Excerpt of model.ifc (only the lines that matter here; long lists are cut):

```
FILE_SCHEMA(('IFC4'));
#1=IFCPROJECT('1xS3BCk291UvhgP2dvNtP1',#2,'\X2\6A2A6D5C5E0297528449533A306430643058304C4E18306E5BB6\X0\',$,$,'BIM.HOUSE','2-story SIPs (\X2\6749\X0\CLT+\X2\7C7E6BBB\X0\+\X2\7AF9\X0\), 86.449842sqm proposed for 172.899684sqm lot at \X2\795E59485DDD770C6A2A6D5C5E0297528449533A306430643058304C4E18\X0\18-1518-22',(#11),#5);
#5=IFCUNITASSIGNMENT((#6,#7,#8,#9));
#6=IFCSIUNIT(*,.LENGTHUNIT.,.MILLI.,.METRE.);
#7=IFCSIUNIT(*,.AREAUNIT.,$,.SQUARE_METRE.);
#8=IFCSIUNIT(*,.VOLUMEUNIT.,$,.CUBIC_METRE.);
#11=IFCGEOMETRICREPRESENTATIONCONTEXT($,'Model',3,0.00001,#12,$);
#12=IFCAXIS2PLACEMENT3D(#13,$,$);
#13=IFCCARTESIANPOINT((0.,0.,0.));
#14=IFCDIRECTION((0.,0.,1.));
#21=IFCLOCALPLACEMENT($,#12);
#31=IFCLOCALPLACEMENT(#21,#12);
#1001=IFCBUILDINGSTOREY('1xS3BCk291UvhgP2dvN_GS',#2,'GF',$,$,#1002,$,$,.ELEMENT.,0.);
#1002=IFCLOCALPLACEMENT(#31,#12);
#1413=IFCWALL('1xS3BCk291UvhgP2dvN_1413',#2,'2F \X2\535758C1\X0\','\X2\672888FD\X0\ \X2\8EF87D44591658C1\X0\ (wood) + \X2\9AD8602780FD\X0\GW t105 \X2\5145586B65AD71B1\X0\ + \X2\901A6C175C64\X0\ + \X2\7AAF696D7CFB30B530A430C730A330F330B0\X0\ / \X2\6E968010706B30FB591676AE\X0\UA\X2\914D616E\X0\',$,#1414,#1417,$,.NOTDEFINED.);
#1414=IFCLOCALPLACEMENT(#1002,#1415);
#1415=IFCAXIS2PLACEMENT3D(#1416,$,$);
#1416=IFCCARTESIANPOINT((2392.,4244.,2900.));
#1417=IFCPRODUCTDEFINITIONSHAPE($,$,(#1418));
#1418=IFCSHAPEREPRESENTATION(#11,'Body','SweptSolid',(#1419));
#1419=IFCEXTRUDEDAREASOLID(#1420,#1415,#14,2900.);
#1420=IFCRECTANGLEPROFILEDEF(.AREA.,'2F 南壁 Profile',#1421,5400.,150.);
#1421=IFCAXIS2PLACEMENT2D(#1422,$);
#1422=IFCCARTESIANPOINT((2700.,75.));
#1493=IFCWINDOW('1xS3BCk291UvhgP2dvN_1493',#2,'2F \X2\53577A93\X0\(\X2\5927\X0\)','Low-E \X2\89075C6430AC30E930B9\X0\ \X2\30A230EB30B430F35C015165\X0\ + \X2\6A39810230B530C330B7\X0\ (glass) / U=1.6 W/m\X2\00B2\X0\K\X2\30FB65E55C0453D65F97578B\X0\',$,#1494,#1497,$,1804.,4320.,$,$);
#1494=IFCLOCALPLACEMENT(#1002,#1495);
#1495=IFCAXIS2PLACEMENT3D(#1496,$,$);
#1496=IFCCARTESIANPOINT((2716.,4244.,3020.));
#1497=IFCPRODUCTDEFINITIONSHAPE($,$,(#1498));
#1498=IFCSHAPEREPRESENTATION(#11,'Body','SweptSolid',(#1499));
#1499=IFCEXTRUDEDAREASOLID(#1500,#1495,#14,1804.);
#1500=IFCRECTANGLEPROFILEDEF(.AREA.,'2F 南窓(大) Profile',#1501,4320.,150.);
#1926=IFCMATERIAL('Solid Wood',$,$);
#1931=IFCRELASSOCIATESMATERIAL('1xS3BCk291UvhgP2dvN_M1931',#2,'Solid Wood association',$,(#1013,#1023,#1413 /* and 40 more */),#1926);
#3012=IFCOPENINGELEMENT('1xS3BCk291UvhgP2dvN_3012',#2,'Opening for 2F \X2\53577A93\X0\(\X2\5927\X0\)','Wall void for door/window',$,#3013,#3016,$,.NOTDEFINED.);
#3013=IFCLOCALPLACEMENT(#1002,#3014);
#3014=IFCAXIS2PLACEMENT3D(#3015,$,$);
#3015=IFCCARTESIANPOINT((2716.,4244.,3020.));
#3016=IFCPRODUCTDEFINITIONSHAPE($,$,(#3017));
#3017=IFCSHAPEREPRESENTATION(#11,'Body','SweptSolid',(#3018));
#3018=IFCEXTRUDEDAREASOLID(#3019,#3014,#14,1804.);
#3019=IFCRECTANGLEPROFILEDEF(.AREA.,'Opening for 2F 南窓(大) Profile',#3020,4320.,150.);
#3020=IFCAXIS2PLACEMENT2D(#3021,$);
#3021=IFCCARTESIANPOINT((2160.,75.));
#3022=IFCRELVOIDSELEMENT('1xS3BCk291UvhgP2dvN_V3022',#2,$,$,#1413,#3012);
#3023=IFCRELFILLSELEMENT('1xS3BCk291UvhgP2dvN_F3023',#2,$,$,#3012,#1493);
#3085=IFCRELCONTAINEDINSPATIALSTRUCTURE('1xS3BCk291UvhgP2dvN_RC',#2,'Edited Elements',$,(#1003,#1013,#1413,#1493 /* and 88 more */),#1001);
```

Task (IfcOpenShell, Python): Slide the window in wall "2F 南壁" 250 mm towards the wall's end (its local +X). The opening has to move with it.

```python
import ifcopenshell
import ifcopenshell.api.geometry
import ifcopenshell.util.placement
import ifcopenshell.util.unit

model = ifcopenshell.open("model.ifc")
unit_scale = ifcopenshell.util.unit.calculate_unit_scale(model)

window = model.by_guid("1xS3BCk291UvhgP2dvN_1493")
opening = window.FillsVoids[0].RelatingOpeningElement
wall = opening.VoidsElements[0].RelatingBuildingElement

wall_matrix = ifcopenshell.util.placement.get_local_placement(wall.ObjectPlacement)
shift = wall_matrix[:3, 0] * 0.25 / unit_scale
before = ifcopenshell.util.placement.get_local_placement(window.ObjectPlacement)[:3, 3].copy()

# The window is not placed relative to its opening, so move both.
for product in (opening, window):
    matrix = ifcopenshell.util.placement.get_local_placement(product.ObjectPlacement)
    matrix[:3, 3] += shift
    ifcopenshell.api.geometry.edit_object_placement(model, product=product, matrix=matrix, is_si=False)

after = ifcopenshell.util.placement.get_local_placement(window.ObjectPlacement)[:3, 3]
print("window moved by", (after - before).round(3) + 0.0)

model.write("model_edited.ifc")
```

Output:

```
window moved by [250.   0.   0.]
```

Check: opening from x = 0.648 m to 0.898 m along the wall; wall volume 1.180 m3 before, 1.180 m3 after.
